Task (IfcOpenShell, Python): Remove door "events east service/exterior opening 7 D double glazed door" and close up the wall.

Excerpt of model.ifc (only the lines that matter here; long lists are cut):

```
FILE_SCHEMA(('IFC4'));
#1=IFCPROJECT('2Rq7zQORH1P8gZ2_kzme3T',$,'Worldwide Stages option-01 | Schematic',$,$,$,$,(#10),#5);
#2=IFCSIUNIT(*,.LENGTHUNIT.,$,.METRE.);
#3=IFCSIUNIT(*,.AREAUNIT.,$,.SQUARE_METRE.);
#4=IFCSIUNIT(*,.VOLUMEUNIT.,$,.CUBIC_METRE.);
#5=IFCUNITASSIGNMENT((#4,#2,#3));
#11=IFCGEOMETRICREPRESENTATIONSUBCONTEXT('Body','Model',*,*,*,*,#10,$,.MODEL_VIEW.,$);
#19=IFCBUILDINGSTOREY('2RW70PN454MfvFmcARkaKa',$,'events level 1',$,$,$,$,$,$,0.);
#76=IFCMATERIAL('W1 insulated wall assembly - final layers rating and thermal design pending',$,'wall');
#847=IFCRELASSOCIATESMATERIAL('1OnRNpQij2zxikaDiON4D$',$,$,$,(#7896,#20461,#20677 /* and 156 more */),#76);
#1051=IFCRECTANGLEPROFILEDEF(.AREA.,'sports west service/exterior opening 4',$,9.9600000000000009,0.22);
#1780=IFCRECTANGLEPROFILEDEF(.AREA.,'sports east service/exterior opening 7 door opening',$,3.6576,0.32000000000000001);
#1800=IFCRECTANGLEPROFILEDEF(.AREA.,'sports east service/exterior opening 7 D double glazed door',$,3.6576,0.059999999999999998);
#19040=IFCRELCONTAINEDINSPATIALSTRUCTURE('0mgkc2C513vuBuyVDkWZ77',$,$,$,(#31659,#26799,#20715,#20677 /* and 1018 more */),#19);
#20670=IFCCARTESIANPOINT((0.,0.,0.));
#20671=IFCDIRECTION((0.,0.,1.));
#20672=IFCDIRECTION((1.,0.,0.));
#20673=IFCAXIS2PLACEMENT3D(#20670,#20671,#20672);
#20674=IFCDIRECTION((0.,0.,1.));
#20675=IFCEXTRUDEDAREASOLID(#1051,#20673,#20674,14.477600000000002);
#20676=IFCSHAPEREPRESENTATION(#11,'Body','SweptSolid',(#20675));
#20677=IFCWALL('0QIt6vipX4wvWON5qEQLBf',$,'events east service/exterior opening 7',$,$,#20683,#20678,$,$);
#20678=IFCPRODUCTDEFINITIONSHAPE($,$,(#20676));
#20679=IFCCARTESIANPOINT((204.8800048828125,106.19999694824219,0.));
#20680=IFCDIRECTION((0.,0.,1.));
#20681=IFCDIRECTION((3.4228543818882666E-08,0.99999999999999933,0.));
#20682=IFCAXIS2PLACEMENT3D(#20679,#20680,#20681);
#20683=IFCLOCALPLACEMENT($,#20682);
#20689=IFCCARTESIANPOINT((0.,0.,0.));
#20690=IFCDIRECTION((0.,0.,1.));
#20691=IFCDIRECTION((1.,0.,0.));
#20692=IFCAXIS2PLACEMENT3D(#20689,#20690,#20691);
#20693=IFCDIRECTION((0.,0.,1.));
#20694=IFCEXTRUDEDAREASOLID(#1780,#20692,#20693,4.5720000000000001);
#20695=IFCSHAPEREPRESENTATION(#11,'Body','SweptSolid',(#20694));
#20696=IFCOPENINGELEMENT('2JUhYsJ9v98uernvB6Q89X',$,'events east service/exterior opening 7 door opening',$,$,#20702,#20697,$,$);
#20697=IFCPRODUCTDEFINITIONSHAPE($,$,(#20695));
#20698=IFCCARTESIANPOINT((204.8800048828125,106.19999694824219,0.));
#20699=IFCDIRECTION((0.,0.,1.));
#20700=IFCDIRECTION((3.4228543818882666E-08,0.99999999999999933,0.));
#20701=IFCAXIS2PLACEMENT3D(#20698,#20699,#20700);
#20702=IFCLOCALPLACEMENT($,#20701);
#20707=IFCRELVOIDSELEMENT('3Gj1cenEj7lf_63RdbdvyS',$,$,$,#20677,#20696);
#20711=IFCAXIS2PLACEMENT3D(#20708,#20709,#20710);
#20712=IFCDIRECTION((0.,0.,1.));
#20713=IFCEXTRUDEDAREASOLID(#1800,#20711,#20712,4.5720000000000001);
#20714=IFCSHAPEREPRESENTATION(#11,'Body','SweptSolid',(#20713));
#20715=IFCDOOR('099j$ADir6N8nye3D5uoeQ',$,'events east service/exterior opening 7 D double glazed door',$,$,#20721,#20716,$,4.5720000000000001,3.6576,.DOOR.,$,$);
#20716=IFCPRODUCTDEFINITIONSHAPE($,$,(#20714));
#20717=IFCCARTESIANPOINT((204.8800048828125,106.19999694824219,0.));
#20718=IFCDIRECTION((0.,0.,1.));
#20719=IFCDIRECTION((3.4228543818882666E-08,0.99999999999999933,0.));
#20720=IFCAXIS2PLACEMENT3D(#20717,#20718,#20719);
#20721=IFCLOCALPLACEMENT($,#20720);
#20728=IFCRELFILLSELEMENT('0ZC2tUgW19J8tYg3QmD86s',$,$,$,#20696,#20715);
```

```python
import ifcopenshell
import ifcopenshell.api.feature
import ifcopenshell.api.root
import ifcopenshell.geom
import ifcopenshell.util.shape

model = ifcopenshell.open("model.ifc")
settings = ifcopenshell.geom.settings()


def volume(element):
    """Net volume in cubic metres, openings subtracted."""
    shape = ifcopenshell.geom.create_shape(settings, element)
    return ifcopenshell.util.shape.get_volume(shape.geometry)


door = model.by_id(20715)
opening = door.FillsVoids[0].RelatingOpeningElement
wall = opening.VoidsElements[0].RelatingBuildingElement
before = volume(wall)

ifcopenshell.api.root.remove_product(model, product=door)
ifcopenshell.api.feature.remove_feature(model, feature=opening)

after = volume(wall)

print(f"wall volume {before:.3f} -> {after:.3f} m3")

model.write("model-out.ifc")
```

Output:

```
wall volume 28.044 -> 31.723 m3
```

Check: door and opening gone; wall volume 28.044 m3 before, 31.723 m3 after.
